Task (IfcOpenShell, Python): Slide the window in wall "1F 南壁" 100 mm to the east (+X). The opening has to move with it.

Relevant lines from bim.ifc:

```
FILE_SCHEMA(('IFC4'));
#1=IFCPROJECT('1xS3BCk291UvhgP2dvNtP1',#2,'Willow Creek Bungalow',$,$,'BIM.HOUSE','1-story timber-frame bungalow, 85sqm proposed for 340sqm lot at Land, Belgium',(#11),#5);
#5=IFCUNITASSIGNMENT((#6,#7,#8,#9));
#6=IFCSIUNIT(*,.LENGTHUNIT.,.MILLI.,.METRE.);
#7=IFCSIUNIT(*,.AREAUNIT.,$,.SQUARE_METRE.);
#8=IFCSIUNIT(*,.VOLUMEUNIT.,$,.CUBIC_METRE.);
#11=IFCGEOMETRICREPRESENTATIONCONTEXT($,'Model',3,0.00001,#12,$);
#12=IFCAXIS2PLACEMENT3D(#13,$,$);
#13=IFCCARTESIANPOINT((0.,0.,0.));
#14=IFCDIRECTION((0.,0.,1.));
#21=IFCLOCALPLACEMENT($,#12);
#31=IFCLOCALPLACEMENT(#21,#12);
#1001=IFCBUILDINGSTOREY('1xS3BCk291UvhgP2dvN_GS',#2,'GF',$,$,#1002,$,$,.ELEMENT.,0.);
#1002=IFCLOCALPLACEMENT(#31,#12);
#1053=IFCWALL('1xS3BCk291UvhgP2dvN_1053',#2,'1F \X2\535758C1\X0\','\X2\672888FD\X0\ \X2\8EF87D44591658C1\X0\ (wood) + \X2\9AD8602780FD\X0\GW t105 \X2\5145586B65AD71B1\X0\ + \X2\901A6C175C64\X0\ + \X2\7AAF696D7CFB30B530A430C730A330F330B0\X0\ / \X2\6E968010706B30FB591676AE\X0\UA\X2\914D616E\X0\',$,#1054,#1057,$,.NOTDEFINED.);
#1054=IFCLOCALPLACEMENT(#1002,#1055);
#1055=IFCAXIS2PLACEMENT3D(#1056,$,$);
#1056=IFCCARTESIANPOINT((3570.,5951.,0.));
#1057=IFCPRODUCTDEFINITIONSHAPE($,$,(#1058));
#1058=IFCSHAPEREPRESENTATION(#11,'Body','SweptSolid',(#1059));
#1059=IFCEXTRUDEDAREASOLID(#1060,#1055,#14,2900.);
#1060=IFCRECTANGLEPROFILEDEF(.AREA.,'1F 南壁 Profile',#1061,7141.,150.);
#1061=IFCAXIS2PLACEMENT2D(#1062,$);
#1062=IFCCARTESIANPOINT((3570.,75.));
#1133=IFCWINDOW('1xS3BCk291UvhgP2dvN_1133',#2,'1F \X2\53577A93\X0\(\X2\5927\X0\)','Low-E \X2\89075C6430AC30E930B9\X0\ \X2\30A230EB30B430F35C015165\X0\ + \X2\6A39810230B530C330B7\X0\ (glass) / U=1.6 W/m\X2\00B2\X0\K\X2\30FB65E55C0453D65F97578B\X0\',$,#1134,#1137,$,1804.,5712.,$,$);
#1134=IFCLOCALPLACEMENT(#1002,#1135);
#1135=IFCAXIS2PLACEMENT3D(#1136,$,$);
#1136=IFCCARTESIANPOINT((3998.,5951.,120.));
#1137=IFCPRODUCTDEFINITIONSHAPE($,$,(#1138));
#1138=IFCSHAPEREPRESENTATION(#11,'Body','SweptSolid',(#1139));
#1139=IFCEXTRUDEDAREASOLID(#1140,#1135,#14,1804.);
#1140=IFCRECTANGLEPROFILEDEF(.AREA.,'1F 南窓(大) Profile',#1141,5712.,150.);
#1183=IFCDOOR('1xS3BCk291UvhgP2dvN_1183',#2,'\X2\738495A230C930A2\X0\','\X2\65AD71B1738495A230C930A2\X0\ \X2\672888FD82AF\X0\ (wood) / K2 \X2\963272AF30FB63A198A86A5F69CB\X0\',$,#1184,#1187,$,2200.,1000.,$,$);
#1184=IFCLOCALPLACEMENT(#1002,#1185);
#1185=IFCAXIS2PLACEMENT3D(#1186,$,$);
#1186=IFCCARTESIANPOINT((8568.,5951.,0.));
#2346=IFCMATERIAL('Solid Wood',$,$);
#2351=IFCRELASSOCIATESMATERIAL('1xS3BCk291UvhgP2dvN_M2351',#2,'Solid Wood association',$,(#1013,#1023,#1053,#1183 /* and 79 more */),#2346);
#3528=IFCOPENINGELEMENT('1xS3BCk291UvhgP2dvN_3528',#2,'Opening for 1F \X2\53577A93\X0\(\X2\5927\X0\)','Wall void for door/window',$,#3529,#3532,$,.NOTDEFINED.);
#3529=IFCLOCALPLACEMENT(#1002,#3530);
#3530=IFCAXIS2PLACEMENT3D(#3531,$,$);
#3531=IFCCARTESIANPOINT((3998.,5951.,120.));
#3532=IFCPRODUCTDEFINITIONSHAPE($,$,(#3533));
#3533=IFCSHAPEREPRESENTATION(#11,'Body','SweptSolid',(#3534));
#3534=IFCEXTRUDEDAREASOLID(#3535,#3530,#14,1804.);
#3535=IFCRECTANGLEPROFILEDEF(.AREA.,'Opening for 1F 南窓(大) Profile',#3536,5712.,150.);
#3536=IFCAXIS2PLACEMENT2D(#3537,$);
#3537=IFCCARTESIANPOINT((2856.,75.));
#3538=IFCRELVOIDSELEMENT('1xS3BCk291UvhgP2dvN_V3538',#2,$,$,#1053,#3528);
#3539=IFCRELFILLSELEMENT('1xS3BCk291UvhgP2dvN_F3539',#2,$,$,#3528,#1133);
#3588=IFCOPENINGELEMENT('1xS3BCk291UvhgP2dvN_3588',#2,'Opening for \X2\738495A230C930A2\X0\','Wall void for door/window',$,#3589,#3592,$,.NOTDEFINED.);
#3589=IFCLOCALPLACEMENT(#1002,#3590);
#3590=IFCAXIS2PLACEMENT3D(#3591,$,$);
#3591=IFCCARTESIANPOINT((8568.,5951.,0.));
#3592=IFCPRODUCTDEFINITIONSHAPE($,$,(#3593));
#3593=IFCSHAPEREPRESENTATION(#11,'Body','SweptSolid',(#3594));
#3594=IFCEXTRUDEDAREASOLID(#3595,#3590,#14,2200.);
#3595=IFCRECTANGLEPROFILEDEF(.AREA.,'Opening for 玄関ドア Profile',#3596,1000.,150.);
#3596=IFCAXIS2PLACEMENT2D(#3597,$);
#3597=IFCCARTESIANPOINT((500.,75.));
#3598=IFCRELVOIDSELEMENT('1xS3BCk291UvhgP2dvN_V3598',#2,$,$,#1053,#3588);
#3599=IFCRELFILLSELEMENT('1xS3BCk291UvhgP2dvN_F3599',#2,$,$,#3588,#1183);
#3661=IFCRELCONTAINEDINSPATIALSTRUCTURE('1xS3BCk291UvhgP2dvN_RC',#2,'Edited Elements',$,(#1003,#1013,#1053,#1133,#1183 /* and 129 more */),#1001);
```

```python
import ifcopenshell
import ifcopenshell.api.geometry
import ifcopenshell.util.placement

model = ifcopenshell.open("bim.ifc")

window = model.by_guid("1xS3BCk291UvhgP2dvN_1133")
opening = window.FillsVoids[0].RelatingOpeningElement
wall = opening.VoidsElements[0].RelatingBuildingElement

wall_matrix = ifcopenshell.util.placement.get_local_placement(wall.ObjectPlacement)
shift = wall_matrix[:3, 0] * 100.0
before = ifcopenshell.util.placement.get_local_placement(window.ObjectPlacement)[:3, 3].copy()

# The window is not placed relative to its opening, so move both.
for product in (opening, window):
    matrix = ifcopenshell.util.placement.get_local_placement(product.ObjectPlacement)
    matrix[:3, 3] += shift
    ifcopenshell.api.geometry.edit_object_placement(model, product=product, matrix=matrix, is_si=False)

after = ifcopenshell.util.placement.get_local_placement(window.ObjectPlacement)[:3, 3]
print("window moved by", (after - before).round(3) + 0.0)

model.write("bim_rev.ifc")
```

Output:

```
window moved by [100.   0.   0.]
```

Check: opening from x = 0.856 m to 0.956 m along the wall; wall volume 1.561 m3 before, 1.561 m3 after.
